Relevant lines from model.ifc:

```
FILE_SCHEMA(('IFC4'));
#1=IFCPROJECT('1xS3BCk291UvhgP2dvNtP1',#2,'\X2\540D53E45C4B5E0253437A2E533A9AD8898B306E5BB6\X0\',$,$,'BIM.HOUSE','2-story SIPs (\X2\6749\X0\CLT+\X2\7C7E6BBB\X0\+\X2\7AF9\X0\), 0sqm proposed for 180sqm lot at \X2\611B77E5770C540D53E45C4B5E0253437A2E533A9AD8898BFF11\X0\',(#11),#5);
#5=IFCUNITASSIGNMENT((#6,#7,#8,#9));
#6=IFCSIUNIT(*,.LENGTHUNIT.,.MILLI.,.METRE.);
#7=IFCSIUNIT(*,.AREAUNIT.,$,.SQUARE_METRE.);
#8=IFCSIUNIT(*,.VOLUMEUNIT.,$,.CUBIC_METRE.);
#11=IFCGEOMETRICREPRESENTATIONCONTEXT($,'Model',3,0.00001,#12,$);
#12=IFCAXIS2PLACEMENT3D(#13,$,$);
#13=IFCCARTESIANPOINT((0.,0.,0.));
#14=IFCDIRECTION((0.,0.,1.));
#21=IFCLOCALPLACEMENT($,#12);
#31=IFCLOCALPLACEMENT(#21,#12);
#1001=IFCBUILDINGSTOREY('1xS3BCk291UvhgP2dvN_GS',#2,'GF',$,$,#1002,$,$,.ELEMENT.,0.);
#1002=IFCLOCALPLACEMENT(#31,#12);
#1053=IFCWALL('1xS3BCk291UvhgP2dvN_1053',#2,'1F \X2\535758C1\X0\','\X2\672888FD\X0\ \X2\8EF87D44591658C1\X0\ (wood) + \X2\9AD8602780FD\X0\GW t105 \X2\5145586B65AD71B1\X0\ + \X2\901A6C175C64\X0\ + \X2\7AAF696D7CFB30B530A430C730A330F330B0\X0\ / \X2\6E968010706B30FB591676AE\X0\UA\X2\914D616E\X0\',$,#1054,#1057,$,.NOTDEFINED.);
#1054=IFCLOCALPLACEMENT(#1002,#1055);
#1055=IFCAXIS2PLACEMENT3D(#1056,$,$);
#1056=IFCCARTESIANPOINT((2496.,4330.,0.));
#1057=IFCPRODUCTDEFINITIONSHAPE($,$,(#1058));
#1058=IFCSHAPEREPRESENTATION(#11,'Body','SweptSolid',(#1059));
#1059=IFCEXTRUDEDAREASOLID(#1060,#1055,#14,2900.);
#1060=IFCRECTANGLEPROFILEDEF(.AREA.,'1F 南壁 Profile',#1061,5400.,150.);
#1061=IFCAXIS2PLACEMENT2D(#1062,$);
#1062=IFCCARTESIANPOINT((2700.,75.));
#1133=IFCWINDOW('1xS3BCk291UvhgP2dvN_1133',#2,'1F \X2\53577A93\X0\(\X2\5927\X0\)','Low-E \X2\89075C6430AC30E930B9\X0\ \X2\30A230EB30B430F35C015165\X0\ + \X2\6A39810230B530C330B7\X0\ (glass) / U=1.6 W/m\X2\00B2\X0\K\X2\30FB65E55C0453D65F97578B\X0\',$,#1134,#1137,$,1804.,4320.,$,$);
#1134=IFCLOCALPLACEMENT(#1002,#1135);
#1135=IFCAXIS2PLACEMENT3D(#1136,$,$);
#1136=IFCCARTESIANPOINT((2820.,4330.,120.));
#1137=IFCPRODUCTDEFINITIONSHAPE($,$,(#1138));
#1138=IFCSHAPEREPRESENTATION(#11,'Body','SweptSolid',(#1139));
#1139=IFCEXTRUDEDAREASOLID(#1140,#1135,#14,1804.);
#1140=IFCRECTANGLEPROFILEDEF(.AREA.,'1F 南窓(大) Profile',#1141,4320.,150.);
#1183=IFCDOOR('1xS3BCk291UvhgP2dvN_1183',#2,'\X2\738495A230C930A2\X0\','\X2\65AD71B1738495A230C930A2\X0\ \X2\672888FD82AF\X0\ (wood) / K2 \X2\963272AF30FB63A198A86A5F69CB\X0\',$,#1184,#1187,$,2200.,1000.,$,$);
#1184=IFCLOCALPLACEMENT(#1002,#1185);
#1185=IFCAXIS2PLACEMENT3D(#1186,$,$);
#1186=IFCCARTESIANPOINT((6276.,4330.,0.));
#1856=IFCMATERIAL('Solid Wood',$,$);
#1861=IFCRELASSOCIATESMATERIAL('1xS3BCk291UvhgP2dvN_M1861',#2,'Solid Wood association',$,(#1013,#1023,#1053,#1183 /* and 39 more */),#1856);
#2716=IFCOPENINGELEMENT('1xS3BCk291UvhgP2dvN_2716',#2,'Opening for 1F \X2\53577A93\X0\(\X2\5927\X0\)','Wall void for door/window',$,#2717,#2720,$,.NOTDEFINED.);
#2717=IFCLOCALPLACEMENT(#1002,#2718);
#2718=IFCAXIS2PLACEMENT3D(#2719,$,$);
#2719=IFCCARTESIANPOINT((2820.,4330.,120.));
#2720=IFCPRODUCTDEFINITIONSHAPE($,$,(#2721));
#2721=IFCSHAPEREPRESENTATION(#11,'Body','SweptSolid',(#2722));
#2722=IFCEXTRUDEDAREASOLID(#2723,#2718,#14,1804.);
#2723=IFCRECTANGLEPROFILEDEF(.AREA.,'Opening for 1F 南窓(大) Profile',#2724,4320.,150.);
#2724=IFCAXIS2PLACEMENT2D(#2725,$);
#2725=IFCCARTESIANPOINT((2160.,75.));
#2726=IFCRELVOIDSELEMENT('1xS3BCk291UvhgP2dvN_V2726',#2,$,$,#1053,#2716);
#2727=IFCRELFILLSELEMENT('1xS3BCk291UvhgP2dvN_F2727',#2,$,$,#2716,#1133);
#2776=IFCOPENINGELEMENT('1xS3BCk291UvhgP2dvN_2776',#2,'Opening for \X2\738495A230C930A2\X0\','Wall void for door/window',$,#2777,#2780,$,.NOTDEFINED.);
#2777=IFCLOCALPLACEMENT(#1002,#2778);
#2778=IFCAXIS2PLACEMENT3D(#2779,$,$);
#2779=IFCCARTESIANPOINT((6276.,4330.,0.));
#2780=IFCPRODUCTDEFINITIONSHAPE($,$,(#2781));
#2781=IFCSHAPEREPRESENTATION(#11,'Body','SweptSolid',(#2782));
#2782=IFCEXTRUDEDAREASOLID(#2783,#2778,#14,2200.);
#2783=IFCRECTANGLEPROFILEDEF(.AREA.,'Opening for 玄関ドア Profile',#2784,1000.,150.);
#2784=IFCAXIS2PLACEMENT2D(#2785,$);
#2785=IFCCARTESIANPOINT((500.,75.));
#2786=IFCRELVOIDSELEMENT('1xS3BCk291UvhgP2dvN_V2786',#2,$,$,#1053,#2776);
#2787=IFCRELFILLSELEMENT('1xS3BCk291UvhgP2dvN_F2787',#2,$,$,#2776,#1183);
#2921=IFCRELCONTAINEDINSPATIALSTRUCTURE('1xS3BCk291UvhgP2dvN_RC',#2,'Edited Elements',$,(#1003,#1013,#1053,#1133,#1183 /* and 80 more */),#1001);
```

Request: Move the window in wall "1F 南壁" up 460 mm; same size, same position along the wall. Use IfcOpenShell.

```python
import numpy as np
import ifcopenshell
import ifcopenshell.api.geometry
import ifcopenshell.util.placement
import ifcopenshell.util.unit

model = ifcopenshell.open("model.ifc")
unit_scale = ifcopenshell.util.unit.calculate_unit_scale(model)

window = model.by_guid("1xS3BCk291UvhgP2dvN_1133")
opening = window.FillsVoids[0].RelatingOpeningElement
dz = 0.46 / unit_scale

shift = np.array([0.0, 0.0, dz])
# The window is not placed relative to its opening, so move both.
for product in (opening, window):
    matrix = ifcopenshell.util.placement.get_local_placement(product.ObjectPlacement)
    matrix[:3, 3] += shift
    ifcopenshell.api.geometry.edit_object_placement(model, product=product, matrix=matrix, is_si=False)

print(f"moved by {dz * unit_scale:+.3f} m")

model.write("model_v2.ifc")
```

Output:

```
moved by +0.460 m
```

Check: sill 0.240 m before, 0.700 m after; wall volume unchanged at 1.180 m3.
